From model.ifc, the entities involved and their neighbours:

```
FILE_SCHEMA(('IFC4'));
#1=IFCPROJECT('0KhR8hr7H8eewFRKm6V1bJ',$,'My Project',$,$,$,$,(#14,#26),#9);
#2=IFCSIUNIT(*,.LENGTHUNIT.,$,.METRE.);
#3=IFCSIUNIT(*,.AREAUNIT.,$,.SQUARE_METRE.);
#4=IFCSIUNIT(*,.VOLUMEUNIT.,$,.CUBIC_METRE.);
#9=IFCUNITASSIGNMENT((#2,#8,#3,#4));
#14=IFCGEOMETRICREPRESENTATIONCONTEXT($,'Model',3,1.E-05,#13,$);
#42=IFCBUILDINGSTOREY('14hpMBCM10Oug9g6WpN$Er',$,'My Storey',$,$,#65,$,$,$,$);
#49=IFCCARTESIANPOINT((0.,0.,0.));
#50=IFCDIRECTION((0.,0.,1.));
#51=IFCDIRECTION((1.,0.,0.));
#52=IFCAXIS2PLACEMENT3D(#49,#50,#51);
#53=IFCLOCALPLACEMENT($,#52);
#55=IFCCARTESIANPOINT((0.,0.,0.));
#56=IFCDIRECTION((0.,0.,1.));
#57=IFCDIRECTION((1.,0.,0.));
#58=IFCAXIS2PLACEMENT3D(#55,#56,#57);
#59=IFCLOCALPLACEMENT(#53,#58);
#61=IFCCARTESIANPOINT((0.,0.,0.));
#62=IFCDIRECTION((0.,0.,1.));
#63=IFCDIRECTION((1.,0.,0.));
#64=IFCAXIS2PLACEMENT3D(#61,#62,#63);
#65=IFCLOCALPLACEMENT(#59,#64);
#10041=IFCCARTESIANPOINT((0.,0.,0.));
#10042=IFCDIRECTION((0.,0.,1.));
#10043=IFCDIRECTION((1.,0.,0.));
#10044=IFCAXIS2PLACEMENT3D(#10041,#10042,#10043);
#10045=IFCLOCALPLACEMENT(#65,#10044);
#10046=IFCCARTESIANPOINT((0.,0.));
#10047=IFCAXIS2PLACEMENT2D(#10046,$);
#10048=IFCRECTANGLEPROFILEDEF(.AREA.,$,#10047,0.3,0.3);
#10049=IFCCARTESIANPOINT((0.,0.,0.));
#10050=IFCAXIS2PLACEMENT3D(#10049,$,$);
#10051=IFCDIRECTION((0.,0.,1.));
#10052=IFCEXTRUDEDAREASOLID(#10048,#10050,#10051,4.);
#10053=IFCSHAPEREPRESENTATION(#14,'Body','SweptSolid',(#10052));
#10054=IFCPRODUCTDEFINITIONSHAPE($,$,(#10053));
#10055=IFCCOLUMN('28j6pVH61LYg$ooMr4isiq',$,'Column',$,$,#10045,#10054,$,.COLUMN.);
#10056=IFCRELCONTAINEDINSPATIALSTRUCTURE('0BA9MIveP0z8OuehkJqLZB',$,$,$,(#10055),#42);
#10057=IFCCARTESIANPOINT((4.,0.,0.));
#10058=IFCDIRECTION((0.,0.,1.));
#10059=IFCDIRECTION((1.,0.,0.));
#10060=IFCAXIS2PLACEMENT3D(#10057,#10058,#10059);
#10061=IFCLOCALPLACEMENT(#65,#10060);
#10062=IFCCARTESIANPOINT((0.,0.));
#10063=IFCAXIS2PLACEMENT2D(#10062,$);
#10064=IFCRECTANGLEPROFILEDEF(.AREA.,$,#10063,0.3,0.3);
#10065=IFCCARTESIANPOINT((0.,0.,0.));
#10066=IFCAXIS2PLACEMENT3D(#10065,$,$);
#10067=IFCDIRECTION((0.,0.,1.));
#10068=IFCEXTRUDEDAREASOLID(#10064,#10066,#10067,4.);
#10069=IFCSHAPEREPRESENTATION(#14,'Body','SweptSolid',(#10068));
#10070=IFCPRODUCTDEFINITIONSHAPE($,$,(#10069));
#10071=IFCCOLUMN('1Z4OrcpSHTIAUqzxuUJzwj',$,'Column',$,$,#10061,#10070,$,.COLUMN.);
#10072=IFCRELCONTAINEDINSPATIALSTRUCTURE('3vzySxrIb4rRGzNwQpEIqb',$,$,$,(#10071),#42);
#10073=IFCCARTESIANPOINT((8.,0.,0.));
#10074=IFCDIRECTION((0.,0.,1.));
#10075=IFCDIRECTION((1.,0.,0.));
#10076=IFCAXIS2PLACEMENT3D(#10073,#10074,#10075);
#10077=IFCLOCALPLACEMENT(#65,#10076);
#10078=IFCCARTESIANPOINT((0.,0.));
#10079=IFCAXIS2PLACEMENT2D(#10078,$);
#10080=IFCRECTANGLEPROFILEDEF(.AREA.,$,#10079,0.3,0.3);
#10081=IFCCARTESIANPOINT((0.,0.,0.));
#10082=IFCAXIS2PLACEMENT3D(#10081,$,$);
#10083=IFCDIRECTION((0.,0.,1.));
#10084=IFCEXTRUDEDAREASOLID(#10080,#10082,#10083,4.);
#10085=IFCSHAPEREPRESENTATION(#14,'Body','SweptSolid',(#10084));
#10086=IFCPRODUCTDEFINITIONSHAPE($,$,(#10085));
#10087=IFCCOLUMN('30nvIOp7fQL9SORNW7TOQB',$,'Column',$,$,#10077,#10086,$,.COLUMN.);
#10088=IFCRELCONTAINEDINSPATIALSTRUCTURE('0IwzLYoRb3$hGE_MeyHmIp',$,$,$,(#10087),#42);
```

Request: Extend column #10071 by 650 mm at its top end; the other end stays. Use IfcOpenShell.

```python
import ifcopenshell
import ifcopenshell.util.unit

model = ifcopenshell.open("model.ifc")
unit_scale = ifcopenshell.util.unit.calculate_unit_scale(model)

member = model.by_guid("1Z4OrcpSHTIAUqzxuUJzwj")
change = 0.65 / unit_scale

# The extrusion runs towards the end named, so only its depth changes.
body = next(r for r in member.Representation.Representations if r.RepresentationIdentifier == "Body")
solid = body.Items[0]
old_length = solid.Depth
solid.Depth += change

print(f"length {old_length:g} -> {solid.Depth:g}")

model.write("model_updated.ifc")
```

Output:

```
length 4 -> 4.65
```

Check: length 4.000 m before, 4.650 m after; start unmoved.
